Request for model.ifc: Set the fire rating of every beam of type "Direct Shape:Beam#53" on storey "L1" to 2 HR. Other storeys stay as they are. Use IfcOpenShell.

First a look at what the model holds.

```python
import ifcopenshell
import ifcopenshell.util.element

model = ifcopenshell.open("model.ifc")
print(model.schema)
storey = next(s for s in model.by_type("IfcBuildingStorey") if s.Name == "L1")
beams = [e for e in ifcopenshell.util.element.get_decomposition(storey) if e.is_a("IfcBeam")]
seen = {}
for e in beams:
    element_type = ifcopenshell.util.element.get_type(e)
    key = (element_type.Name if element_type != e and element_type else None, ifcopenshell.util.element.get_pset(e, "Pset_BeamCommon", "FireRating"))
    seen[key] = seen.get(key, 0) + 1
for (name, value), count in sorted(seen.items(), key=str):
    print(count, "x", name, "|", value)
```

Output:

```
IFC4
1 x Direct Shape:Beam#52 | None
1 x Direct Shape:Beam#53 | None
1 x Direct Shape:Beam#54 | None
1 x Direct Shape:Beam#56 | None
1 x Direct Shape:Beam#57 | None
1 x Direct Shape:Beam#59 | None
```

```python
import ifcopenshell
import ifcopenshell.api.pset
import ifcopenshell.util.element

model = ifcopenshell.open("model.ifc")

storey = next(s for s in model.by_type("IfcBuildingStorey") if s.Name == "L1")
beams = [e for e in ifcopenshell.util.element.get_decomposition(storey) if e.is_a("IfcBeam")]

count = 0
for e in beams:
    element_type = ifcopenshell.util.element.get_type(e)
    if element_type in (None, e) or element_type.Name != "Direct Shape:Beam#53":
        continue
    # add_pset returns the element's existing set when there is one.
    pset = ifcopenshell.api.pset.add_pset(model, product=e, name="Pset_BeamCommon")
    ifcopenshell.api.pset.edit_pset(model, pset=pset, properties={"FireRating": "2 HR"})
    count += 1

print(count, "beams updated")

model.write("model-out.ifc")
```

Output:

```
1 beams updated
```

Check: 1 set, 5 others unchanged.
